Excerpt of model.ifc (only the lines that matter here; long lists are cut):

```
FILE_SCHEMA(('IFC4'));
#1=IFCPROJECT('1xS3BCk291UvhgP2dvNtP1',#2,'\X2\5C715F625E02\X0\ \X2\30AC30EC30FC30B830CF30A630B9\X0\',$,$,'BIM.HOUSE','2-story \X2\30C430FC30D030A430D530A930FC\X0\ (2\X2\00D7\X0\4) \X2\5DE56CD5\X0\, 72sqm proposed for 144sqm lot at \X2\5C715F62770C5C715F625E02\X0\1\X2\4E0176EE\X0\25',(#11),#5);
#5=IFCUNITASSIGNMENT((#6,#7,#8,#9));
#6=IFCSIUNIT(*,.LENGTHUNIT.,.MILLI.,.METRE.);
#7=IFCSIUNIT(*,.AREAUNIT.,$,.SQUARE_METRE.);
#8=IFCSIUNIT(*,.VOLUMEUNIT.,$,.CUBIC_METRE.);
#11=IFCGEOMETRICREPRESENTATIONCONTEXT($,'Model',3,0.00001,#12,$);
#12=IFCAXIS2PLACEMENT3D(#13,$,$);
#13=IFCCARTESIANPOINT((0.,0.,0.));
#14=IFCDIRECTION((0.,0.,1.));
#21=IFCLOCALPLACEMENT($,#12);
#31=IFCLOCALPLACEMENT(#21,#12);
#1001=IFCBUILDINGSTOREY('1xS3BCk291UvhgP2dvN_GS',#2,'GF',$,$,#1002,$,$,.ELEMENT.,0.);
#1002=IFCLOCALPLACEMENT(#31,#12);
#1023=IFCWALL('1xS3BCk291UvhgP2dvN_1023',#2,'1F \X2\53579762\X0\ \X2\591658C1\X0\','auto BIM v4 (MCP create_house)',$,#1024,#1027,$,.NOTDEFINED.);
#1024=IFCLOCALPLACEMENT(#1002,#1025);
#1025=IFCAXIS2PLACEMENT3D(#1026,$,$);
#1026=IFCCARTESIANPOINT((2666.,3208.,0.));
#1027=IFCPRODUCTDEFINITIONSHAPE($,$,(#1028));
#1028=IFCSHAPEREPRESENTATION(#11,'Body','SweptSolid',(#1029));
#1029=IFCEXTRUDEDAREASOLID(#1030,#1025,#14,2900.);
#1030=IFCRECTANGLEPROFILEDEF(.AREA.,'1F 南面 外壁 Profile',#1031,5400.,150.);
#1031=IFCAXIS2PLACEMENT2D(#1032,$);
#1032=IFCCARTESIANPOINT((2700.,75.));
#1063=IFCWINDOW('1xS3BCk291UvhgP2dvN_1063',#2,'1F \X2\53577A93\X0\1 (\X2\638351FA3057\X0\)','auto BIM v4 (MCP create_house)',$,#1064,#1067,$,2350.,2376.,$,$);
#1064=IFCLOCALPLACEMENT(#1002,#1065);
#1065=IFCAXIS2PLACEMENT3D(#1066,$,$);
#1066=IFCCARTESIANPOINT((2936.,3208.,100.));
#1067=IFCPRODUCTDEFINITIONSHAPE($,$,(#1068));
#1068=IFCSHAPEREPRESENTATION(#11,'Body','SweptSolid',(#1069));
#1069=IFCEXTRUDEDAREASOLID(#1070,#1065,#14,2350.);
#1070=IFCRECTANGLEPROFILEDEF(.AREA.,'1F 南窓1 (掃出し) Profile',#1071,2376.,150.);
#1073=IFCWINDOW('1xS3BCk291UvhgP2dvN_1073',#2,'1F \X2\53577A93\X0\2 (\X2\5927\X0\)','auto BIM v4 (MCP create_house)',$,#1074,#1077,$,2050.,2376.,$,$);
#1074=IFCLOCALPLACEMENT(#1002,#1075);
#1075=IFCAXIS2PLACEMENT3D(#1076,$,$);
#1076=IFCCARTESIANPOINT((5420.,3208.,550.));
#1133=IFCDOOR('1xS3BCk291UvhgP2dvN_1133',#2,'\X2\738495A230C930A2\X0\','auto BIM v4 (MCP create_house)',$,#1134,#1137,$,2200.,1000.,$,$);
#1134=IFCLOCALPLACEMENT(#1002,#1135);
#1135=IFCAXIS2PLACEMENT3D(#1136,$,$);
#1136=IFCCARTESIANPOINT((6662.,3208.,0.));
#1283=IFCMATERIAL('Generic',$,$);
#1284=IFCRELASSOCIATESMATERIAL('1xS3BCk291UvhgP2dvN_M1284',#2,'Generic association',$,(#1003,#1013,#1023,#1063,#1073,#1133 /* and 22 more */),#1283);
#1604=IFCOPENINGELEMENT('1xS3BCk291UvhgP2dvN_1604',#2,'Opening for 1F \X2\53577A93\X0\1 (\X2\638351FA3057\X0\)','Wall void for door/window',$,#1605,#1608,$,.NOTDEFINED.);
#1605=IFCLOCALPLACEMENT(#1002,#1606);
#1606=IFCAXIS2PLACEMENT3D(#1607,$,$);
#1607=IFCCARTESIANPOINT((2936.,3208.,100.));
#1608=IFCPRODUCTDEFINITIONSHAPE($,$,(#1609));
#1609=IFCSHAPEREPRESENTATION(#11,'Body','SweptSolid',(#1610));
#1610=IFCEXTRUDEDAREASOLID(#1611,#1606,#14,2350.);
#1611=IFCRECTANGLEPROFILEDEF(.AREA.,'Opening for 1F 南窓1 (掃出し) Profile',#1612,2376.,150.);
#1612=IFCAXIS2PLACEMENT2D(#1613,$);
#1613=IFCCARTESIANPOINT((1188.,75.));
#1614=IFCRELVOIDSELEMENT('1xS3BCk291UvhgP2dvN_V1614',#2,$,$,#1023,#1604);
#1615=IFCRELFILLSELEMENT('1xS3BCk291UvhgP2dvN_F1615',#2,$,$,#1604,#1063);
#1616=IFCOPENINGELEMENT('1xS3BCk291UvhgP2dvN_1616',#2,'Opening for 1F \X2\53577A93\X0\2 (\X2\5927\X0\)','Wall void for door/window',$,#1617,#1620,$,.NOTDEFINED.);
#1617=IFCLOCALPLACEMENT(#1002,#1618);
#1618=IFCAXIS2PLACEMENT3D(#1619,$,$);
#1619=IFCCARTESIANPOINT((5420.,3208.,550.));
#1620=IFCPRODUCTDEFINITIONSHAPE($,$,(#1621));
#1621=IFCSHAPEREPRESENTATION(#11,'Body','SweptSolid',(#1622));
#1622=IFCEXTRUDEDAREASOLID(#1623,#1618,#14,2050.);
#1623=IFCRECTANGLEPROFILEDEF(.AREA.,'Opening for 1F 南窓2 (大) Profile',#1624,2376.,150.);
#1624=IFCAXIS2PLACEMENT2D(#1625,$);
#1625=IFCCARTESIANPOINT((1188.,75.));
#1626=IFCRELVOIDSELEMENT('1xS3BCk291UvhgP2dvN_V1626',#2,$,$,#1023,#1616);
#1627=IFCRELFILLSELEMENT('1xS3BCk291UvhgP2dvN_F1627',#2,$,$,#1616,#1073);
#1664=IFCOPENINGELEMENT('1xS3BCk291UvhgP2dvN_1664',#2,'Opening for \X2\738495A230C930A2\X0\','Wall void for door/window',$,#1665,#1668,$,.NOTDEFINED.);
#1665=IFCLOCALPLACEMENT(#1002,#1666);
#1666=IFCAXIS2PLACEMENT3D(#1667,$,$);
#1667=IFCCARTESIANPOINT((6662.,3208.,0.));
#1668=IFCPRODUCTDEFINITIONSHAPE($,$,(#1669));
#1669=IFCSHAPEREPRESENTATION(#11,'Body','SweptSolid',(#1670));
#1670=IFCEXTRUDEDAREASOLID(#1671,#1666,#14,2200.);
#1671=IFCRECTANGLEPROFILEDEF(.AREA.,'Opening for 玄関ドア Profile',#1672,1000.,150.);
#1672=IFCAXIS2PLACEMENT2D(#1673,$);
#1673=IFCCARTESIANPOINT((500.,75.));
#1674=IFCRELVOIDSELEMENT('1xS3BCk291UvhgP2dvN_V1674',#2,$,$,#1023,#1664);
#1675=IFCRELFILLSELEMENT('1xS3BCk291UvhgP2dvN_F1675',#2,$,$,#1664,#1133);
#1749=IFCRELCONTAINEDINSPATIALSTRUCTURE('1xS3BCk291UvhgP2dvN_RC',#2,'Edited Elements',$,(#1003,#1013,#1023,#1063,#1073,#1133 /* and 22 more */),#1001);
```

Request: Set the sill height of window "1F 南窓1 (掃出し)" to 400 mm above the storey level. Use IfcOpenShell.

```python
import numpy as np
import ifcopenshell
import ifcopenshell.api.geometry
import ifcopenshell.geom
import ifcopenshell.util.element
import ifcopenshell.util.placement
import ifcopenshell.util.shape
import ifcopenshell.util.unit

model = ifcopenshell.open("model.ifc")
unit_scale = ifcopenshell.util.unit.calculate_unit_scale(model)

window = model.by_id(1063)
opening = window.FillsVoids[0].RelatingOpeningElement
storey = ifcopenshell.util.element.get_container(window, ifc_class="IfcBuildingStorey")
level = ifcopenshell.util.placement.get_local_placement(storey.ObjectPlacement)[2, 3]

# The opening's origin need not be at the sill, so measure its lowest point.
shape = ifcopenshell.geom.create_shape(ifcopenshell.geom.settings(), opening)
bottom = ifcopenshell.util.shape.get_shape_bottom_elevation(shape, shape.geometry) / unit_scale
dz = level + 0.4 / unit_scale - bottom

shift = np.array([0.0, 0.0, dz])
# The window is not placed relative to its opening, so move both.
for product in (opening, window):
    matrix = ifcopenshell.util.placement.get_local_placement(product.ObjectPlacement)
    matrix[:3, 3] += shift
    ifcopenshell.api.geometry.edit_object_placement(model, product=product, matrix=matrix, is_si=False)

print(f"moved by {dz * unit_scale:+.3f} m")

model.write("model_updated.ifc")
```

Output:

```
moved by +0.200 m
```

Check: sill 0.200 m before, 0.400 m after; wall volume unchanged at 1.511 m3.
